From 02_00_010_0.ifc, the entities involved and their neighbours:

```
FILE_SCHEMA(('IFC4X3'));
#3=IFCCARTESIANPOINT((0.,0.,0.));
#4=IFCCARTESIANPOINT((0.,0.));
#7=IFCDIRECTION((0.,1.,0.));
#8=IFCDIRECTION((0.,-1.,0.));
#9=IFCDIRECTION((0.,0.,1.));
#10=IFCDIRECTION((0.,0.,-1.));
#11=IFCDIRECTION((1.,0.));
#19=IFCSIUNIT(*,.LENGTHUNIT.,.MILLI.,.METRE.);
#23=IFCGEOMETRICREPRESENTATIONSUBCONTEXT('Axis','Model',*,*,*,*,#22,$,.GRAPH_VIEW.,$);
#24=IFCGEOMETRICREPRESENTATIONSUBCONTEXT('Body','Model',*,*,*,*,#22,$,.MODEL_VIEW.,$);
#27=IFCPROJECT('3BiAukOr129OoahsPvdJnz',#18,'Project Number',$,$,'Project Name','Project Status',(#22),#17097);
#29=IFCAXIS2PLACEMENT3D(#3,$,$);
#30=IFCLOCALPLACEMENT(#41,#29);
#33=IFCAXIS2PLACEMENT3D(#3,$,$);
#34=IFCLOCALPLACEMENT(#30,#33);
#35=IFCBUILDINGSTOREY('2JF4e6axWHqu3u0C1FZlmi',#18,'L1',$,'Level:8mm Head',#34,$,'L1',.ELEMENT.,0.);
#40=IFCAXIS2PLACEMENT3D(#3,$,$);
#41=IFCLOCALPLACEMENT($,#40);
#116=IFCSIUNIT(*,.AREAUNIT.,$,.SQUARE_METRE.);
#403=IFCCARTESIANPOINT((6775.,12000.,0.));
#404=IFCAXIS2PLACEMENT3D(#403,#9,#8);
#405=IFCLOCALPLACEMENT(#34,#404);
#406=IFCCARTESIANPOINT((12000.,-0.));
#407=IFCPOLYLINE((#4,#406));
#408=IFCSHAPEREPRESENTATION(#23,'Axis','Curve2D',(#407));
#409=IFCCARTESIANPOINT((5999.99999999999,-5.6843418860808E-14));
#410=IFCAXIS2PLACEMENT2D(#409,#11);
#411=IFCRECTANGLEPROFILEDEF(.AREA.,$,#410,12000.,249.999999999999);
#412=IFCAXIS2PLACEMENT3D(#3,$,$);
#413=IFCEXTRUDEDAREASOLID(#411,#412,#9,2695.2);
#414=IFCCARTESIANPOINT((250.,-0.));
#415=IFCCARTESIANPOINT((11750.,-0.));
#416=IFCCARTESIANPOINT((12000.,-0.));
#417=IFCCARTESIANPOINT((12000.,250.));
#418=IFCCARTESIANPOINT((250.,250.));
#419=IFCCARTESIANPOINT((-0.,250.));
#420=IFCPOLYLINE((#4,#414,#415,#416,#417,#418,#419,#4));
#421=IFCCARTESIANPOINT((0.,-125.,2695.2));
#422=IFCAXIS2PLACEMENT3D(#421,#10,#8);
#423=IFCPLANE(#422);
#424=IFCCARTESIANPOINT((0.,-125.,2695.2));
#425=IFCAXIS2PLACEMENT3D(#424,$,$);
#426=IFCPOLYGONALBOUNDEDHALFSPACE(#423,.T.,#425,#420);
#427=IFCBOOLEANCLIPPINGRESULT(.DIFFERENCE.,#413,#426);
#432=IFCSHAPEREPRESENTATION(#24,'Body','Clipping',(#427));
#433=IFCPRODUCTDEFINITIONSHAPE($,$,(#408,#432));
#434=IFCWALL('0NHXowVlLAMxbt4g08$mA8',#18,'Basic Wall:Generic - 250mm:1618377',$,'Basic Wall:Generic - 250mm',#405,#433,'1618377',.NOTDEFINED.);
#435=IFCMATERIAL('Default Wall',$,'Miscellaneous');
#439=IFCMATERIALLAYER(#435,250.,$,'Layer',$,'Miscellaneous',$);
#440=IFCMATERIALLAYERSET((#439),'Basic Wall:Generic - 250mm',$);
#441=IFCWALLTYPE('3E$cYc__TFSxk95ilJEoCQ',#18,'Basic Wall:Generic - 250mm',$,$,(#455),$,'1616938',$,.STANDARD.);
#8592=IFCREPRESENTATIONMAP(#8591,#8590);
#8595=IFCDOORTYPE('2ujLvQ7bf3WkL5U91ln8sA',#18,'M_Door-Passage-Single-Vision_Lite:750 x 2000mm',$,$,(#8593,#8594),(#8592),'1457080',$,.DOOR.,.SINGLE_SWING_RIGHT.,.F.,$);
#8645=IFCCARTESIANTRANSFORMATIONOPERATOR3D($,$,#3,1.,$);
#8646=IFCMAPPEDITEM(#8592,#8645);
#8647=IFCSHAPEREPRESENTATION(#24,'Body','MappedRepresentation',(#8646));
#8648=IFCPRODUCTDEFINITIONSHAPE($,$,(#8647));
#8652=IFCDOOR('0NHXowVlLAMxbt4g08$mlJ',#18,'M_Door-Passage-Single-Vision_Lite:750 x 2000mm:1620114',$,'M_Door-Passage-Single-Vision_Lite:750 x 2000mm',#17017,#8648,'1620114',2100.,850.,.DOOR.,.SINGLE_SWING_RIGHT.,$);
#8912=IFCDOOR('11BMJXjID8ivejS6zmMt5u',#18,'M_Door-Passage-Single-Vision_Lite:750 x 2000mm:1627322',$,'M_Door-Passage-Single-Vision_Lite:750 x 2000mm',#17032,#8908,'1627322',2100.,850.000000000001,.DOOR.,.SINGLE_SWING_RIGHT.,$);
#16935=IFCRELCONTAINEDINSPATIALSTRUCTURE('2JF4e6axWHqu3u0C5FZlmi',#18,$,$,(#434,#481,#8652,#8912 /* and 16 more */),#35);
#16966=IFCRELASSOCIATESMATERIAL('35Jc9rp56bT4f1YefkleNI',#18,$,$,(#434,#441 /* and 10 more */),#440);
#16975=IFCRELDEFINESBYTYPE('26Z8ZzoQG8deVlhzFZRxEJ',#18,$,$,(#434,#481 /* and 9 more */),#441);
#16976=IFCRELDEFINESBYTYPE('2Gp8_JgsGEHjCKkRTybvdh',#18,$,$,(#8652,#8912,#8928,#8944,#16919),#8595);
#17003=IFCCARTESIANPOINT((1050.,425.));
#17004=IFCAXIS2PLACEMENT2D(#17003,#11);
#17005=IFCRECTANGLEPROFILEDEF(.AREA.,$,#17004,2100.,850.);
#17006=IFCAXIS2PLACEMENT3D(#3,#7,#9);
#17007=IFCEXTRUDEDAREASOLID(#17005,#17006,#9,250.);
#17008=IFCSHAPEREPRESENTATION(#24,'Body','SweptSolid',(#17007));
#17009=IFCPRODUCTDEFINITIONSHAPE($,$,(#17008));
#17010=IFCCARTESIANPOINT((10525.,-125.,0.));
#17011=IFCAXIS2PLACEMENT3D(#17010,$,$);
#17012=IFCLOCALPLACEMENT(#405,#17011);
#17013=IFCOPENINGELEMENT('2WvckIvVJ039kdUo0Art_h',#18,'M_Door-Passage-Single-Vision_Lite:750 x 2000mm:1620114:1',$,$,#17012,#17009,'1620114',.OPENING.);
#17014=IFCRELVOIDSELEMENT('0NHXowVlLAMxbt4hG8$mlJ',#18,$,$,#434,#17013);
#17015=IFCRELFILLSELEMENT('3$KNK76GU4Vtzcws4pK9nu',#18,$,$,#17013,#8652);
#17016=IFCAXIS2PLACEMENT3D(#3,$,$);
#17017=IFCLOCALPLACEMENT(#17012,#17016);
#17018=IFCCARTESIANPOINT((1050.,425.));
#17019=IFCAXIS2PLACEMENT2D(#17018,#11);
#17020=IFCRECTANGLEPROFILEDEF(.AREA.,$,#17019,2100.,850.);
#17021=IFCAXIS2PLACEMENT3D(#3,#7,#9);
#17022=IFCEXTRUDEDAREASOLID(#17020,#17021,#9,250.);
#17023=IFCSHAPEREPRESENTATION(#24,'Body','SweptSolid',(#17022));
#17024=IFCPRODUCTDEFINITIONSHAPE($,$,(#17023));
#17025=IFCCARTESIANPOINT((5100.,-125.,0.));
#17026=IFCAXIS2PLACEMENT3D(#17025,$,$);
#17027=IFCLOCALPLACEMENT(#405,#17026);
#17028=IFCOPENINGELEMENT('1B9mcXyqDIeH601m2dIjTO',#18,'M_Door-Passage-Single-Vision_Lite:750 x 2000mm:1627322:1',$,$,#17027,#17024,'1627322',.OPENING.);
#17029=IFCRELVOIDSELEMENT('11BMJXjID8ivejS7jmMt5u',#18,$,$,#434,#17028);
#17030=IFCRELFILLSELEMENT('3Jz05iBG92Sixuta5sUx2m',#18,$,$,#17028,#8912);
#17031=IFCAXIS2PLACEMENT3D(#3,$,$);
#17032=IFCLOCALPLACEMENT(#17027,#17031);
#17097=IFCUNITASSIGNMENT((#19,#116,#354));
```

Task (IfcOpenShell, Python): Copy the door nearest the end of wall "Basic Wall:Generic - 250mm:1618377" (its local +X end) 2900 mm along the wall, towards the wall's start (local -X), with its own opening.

```python
import ifcopenshell
import ifcopenshell.api.feature
import ifcopenshell.api.geometry
import ifcopenshell.api.root
import ifcopenshell.geom
import ifcopenshell.util.element
import ifcopenshell.util.placement
import ifcopenshell.util.shape
import ifcopenshell.util.unit

model = ifcopenshell.open("02_00_010_0.ifc")
unit_scale = ifcopenshell.util.unit.calculate_unit_scale(model)
settings = ifcopenshell.geom.settings()


def volume(element):
    """Net volume in cubic metres, openings subtracted."""
    shape = ifcopenshell.geom.create_shape(settings, element)
    return ifcopenshell.util.shape.get_volume(shape.geometry)


def reuse_history(source, copy):
    """copy_class also copies each property set's owner history, people and application; keep the originals."""
    for rel in copy.IsDefinedBy:
        if rel.is_a("IfcRelDefinesByProperties") and (history := rel.RelatingPropertyDefinition.OwnerHistory):
            rel.RelatingPropertyDefinition.OwnerHistory = source.OwnerHistory
            ifcopenshell.util.element.remove_deep2(model, history)


door = model.by_guid("0NHXowVlLAMxbt4g08$mlJ")
opening = door.FillsVoids[0].RelatingOpeningElement
wall = opening.VoidsElements[0].RelatingBuildingElement
before = volume(wall)
shift = ifcopenshell.util.placement.get_local_placement(wall.ObjectPlacement)[:3, 0] * -2.9 / unit_scale

# copy_class copies the void relationship, type, container and properties, but no geometry.
new_opening = ifcopenshell.api.root.copy_class(model, product=opening)
new_opening.Representation = ifcopenshell.util.element.copy_deep(
    model, opening.Representation, exclude=["IfcGeometricRepresentationContext", "IfcRepresentationMap"]
)
new_opening.Name = "M_Door-Passage-Single-Vision_Lite:750 x 2000mm"
new_opening.Tag = None
new_door = ifcopenshell.api.root.copy_class(model, product=door)
new_door.Representation = ifcopenshell.util.element.copy_deep(
    model, door.Representation, exclude=["IfcGeometricRepresentationContext", "IfcRepresentationMap"]
)
new_door.Name = "M_Door-Passage-Single-Vision_Lite:750 x 2000mm"
new_door.Tag = None
reuse_history(door, new_door)
ifcopenshell.api.feature.add_filling(model, opening=new_opening, element=new_door)

for old, new in ((opening, new_opening), (door, new_door)):
    matrix = ifcopenshell.util.placement.get_local_placement(old.ObjectPlacement)
    matrix[:3, 3] += shift
    ifcopenshell.api.geometry.edit_object_placement(model, product=new, matrix=matrix, is_si=False)

after = volume(wall)

print(f"wall volume {before:.3f} -> {after:.3f} m3")

model.write("02_00_010_0_rev.ifc")
```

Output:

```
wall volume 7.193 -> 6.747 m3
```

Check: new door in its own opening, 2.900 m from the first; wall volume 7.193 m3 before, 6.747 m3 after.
